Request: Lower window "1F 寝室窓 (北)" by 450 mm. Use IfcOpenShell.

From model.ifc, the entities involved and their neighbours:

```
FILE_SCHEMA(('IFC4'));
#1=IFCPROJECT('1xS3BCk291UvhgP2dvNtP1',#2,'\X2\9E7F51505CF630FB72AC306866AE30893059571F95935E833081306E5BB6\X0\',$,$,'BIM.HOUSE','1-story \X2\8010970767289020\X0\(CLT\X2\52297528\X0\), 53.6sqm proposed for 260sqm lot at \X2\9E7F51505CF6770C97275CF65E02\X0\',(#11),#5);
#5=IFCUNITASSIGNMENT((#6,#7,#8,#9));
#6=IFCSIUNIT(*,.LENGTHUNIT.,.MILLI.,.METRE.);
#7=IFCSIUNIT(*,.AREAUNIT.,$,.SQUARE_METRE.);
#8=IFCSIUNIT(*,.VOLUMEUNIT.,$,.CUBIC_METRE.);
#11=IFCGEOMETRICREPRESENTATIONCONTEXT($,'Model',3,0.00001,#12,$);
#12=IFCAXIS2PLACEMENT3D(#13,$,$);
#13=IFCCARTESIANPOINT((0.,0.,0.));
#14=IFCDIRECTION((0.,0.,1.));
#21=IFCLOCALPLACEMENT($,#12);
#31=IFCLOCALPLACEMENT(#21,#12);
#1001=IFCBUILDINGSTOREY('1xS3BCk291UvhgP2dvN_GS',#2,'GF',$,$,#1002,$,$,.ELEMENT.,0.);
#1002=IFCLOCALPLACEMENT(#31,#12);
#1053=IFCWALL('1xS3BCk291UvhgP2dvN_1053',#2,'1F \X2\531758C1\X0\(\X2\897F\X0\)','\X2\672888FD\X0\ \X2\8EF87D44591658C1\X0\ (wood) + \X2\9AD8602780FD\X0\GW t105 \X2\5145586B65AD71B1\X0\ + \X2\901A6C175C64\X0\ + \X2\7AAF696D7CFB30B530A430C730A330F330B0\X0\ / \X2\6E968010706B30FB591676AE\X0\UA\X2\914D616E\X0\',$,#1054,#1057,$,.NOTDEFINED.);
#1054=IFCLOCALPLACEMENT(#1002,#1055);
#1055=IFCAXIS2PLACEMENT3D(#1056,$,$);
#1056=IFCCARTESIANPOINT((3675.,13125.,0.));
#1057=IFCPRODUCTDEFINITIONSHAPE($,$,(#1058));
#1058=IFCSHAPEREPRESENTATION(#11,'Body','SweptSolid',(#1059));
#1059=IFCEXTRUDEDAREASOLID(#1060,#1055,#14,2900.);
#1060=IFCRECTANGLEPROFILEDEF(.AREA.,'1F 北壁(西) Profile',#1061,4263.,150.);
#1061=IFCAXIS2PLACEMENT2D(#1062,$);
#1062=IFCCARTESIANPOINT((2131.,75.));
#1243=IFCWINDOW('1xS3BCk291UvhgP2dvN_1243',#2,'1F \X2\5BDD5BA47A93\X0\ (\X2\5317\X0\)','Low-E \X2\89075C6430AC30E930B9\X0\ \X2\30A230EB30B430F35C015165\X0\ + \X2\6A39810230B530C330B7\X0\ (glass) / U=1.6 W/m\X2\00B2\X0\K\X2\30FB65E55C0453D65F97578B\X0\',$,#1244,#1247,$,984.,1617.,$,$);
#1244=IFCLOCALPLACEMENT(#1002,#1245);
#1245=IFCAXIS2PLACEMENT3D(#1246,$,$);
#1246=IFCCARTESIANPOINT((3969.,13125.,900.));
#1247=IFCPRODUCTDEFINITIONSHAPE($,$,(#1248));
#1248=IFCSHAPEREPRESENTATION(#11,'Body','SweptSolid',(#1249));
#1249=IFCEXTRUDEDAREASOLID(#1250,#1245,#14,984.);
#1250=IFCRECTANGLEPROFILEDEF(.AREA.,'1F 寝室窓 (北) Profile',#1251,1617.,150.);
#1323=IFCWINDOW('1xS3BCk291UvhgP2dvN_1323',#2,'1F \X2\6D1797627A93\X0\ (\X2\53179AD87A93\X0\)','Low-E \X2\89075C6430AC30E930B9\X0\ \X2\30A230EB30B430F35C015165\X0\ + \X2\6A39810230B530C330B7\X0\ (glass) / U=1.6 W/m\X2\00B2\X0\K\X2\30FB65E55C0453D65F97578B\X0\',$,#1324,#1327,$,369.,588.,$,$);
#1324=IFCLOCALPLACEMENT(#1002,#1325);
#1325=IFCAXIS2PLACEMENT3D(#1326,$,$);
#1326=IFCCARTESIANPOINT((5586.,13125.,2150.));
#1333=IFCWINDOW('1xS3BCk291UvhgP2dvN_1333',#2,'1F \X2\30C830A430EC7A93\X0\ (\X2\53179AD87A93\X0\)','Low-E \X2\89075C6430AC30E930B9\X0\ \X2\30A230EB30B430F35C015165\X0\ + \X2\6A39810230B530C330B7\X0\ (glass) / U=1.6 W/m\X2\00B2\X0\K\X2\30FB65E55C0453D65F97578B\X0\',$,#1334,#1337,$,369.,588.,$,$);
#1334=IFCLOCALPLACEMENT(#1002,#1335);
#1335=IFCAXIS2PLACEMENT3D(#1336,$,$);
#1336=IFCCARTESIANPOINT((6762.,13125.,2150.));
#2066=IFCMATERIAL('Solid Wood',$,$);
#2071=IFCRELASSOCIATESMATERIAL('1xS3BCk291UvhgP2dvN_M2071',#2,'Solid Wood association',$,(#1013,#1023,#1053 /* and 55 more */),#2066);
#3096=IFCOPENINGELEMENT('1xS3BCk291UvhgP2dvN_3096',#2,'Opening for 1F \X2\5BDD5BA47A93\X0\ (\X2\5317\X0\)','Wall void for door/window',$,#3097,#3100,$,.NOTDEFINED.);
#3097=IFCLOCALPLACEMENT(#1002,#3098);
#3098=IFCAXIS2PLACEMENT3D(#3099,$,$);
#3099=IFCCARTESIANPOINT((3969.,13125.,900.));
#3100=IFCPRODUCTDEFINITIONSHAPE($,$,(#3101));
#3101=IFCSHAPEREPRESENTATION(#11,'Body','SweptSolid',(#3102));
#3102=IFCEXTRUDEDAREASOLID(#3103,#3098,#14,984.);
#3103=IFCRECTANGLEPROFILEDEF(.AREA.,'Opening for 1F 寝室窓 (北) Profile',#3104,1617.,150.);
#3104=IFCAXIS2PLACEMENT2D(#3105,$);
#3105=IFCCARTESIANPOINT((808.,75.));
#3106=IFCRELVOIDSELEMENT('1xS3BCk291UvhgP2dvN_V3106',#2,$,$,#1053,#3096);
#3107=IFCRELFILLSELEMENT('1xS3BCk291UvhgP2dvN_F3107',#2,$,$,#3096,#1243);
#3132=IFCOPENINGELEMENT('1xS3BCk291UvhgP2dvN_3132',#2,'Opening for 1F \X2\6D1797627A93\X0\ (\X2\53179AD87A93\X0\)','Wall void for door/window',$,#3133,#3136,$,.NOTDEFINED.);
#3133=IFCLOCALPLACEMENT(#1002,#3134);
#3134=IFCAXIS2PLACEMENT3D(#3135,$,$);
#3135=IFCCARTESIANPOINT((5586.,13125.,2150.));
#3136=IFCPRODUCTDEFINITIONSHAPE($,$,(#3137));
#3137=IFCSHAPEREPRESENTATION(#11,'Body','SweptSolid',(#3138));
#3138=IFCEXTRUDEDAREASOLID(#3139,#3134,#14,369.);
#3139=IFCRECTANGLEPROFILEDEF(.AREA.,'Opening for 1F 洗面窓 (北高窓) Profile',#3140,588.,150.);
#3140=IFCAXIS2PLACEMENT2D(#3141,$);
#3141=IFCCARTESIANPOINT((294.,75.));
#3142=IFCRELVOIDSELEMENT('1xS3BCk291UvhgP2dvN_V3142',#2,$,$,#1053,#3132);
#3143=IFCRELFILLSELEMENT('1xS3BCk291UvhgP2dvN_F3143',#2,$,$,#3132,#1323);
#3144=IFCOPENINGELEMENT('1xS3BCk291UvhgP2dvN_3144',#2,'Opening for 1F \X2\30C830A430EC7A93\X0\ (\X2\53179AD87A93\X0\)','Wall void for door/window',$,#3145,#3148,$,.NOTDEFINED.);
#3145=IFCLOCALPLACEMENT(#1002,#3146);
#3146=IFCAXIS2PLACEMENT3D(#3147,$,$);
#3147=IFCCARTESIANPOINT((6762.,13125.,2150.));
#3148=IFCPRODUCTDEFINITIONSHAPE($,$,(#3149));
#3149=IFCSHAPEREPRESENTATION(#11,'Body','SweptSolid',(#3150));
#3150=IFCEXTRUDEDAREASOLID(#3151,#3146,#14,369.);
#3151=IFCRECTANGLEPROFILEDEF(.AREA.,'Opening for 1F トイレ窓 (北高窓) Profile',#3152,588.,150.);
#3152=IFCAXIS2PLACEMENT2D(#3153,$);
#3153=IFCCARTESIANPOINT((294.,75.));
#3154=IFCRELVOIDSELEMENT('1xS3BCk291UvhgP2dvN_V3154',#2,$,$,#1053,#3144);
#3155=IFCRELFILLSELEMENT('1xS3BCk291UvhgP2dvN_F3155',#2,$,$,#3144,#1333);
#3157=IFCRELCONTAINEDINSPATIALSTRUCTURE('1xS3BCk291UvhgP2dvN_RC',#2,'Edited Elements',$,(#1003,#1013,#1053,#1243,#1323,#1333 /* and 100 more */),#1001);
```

```python
import numpy as np
import ifcopenshell
import ifcopenshell.api.geometry
import ifcopenshell.util.placement
import ifcopenshell.util.unit

model = ifcopenshell.open("model.ifc")
unit_scale = ifcopenshell.util.unit.calculate_unit_scale(model)

window = model.by_id(1243)
opening = window.FillsVoids[0].RelatingOpeningElement
dz = -450.0

shift = np.array([0.0, 0.0, dz])
# The window is not placed relative to its opening, so move both.
for product in (opening, window):
    matrix = ifcopenshell.util.placement.get_local_placement(product.ObjectPlacement)
    matrix[:3, 3] += shift
    ifcopenshell.api.geometry.edit_object_placement(model, product=product, matrix=matrix, is_si=False)

print(f"moved by {dz * unit_scale:+.3f} m")

model.write("model_rev.ifc")
```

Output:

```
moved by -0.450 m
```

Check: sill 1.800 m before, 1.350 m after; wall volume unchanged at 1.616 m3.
